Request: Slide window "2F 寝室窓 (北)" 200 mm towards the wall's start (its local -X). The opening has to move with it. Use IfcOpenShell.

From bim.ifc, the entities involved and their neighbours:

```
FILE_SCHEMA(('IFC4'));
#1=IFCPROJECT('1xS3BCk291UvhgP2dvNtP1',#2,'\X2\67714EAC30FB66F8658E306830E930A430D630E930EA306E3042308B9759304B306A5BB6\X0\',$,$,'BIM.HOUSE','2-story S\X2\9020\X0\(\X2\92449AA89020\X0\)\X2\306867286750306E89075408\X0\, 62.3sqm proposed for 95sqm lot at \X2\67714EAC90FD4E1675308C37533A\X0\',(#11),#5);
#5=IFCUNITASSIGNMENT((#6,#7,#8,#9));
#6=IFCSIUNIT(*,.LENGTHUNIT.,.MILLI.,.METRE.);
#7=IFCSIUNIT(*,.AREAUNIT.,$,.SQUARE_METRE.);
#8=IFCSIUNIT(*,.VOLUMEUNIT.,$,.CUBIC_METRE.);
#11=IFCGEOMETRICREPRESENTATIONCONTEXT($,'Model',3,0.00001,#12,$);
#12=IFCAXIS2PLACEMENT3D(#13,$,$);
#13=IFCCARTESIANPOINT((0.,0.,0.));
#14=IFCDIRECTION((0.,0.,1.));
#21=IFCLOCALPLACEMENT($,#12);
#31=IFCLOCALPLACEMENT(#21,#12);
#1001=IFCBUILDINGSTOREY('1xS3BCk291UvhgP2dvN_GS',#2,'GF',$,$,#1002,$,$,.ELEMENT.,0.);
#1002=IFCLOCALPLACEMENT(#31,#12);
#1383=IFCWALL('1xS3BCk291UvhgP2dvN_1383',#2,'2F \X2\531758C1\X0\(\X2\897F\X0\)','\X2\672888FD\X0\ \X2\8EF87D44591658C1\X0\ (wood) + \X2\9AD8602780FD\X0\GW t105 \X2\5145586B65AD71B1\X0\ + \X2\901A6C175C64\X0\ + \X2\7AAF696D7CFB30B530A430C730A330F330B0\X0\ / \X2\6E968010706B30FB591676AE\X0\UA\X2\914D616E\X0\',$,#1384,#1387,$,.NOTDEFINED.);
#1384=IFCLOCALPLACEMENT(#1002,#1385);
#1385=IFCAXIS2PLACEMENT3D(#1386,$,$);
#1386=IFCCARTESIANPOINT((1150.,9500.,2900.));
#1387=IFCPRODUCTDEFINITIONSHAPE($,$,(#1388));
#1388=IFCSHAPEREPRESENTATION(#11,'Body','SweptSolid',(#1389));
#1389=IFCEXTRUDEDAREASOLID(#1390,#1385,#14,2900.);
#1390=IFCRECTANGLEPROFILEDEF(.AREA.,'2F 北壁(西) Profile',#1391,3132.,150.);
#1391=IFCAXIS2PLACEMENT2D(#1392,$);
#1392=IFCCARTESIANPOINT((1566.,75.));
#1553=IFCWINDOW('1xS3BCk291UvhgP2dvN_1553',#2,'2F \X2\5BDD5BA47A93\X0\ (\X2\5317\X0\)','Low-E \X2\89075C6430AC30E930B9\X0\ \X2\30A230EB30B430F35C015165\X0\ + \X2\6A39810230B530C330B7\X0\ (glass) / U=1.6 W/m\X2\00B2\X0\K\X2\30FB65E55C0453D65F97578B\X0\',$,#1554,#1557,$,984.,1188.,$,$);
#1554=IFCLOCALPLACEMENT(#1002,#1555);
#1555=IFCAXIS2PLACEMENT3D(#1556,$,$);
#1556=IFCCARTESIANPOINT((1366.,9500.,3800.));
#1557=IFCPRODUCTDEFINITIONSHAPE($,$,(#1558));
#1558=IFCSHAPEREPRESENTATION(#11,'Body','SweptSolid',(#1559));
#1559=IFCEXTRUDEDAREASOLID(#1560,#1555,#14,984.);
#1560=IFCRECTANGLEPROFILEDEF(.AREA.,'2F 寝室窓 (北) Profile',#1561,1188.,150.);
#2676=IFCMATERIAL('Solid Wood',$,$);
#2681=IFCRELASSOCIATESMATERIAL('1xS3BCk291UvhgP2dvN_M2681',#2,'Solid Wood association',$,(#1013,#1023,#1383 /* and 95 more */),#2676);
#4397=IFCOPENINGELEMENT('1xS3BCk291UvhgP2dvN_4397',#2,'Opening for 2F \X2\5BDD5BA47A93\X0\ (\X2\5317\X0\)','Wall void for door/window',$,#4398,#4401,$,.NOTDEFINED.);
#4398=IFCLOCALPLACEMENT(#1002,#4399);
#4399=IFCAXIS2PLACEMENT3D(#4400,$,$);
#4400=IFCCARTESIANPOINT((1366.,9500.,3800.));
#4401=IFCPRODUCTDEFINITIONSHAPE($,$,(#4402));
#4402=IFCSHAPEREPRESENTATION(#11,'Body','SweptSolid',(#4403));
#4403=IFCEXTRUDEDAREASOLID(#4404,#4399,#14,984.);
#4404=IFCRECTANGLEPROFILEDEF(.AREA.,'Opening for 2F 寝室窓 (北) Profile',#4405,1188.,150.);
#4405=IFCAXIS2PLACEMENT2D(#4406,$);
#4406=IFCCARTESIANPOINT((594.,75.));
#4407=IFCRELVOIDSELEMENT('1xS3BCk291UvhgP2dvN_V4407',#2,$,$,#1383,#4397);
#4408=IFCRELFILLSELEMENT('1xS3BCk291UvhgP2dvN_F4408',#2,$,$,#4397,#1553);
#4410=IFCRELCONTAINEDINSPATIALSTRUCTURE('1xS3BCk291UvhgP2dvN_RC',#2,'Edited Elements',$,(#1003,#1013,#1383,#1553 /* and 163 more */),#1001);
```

```python
import ifcopenshell
import ifcopenshell.api.geometry
import ifcopenshell.util.placement

model = ifcopenshell.open("bim.ifc")

window = model.by_id(1553)
opening = window.FillsVoids[0].RelatingOpeningElement
wall = opening.VoidsElements[0].RelatingBuildingElement

wall_matrix = ifcopenshell.util.placement.get_local_placement(wall.ObjectPlacement)
shift = wall_matrix[:3, 0] * -200.0
before = ifcopenshell.util.placement.get_local_placement(window.ObjectPlacement)[:3, 3].copy()

# The window is not placed relative to its opening, so move both.
for product in (opening, window):
    matrix = ifcopenshell.util.placement.get_local_placement(product.ObjectPlacement)
    matrix[:3, 3] += shift
    ifcopenshell.api.geometry.edit_object_placement(model, product=product, matrix=matrix, is_si=False)

after = ifcopenshell.util.placement.get_local_placement(window.ObjectPlacement)[:3, 3]
print("window moved by", (after - before).round(3) + 0.0)

model.write("bim_updated.ifc")
```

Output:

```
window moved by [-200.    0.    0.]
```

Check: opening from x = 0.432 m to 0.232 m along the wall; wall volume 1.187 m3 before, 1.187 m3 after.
